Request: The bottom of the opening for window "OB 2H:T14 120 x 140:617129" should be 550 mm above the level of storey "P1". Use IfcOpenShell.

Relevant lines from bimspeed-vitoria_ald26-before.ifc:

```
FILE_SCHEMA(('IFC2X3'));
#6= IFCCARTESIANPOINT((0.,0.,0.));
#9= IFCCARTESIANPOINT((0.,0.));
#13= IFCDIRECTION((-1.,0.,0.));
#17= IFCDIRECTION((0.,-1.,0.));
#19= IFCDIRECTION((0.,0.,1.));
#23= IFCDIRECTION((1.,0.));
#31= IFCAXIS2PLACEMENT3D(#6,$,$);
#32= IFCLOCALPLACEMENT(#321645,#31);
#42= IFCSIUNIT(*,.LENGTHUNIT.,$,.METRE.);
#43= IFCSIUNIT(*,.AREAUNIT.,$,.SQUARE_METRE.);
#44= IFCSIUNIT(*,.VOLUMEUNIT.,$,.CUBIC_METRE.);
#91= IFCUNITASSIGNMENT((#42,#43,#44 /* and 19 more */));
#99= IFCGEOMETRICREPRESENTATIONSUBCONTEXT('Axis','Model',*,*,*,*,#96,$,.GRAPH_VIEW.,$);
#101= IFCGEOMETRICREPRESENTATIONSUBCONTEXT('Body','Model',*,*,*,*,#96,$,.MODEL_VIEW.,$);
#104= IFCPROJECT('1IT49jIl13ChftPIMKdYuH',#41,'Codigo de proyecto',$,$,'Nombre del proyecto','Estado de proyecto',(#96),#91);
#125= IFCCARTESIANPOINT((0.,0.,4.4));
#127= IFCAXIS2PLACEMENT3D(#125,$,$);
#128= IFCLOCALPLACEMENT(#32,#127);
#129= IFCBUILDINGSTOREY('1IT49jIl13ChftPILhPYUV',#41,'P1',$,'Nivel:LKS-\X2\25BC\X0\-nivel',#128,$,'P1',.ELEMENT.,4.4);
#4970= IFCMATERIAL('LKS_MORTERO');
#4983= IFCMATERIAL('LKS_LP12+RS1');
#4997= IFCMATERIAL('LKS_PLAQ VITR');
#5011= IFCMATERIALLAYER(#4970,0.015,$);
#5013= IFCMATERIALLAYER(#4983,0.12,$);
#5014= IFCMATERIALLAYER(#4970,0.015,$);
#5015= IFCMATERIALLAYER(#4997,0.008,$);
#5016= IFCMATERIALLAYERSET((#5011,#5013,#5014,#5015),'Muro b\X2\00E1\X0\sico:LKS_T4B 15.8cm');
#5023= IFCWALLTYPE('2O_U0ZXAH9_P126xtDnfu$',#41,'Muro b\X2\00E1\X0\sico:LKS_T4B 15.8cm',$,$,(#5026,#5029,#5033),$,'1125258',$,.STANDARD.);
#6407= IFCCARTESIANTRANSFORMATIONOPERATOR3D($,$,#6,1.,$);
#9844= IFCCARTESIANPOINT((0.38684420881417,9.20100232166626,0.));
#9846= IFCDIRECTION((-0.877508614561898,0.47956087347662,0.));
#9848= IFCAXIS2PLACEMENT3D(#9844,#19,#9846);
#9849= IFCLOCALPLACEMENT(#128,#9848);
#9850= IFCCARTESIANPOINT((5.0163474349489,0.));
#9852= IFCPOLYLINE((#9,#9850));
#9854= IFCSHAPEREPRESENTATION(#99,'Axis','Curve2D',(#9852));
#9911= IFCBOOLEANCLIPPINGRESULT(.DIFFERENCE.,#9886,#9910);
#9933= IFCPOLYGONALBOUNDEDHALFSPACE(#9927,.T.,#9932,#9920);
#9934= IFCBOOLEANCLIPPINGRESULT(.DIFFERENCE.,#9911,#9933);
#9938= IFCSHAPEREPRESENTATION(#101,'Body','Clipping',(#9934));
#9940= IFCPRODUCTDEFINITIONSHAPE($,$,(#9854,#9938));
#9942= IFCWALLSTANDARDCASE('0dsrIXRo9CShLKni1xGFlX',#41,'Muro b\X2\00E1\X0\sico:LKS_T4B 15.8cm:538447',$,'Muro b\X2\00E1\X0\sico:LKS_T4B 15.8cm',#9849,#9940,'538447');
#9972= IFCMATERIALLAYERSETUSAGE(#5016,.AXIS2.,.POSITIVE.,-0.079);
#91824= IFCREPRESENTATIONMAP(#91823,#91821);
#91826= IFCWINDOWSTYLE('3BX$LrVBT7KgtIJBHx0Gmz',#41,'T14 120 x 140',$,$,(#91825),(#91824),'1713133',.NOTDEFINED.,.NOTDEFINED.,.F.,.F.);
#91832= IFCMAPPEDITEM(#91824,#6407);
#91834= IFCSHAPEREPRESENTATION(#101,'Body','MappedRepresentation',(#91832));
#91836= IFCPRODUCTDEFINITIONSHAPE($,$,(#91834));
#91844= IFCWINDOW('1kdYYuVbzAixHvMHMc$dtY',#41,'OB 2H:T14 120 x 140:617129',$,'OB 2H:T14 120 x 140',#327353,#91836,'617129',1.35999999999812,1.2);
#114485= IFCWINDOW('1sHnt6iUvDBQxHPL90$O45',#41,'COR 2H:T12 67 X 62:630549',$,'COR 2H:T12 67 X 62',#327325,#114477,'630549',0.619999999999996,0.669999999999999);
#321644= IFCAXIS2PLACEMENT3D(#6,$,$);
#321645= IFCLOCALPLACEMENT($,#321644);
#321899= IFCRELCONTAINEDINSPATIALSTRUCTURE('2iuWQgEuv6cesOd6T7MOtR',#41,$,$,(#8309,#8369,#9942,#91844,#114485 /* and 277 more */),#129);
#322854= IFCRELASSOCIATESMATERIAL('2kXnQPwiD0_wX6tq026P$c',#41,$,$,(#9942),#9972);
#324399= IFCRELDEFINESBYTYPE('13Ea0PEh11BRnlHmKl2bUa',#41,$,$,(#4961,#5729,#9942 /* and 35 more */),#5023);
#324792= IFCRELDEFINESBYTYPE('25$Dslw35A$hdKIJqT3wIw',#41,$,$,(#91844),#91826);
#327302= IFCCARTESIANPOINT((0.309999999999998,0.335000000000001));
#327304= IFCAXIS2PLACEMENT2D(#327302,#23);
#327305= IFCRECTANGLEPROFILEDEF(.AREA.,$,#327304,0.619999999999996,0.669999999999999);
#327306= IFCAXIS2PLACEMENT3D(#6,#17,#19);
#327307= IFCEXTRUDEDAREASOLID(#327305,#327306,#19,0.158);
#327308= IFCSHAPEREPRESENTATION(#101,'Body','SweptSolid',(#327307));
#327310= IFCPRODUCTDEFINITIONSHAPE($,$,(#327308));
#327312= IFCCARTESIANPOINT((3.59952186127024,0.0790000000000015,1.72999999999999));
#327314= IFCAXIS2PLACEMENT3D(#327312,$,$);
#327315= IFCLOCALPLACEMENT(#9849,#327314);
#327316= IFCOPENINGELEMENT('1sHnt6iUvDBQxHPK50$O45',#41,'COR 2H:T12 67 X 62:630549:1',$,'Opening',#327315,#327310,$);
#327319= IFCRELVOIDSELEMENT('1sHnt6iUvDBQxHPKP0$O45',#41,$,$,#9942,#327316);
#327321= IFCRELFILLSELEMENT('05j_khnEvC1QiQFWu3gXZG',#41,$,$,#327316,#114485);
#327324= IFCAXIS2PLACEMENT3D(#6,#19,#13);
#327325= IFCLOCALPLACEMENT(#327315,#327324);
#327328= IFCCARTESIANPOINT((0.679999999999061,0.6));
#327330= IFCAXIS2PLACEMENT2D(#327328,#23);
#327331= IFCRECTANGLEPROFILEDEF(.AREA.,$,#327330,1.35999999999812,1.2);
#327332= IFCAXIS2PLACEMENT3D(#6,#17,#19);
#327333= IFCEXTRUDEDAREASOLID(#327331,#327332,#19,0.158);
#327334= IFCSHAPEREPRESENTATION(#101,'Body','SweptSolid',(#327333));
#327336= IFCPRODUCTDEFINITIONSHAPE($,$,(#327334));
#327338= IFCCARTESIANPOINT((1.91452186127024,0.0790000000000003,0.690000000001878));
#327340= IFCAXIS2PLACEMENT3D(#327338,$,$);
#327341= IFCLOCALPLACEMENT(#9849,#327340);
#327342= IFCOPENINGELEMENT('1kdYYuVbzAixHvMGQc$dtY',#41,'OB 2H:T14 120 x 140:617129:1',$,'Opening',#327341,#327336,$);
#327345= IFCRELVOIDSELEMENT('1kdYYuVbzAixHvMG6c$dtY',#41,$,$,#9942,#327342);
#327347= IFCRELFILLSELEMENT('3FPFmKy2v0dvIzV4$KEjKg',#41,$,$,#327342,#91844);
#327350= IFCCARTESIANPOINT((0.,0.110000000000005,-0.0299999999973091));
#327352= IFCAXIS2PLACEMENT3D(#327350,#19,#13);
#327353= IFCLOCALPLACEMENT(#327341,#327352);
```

```python
import numpy as np
import ifcopenshell
import ifcopenshell.api.geometry
import ifcopenshell.geom
import ifcopenshell.util.element
import ifcopenshell.util.placement
import ifcopenshell.util.shape
import ifcopenshell.util.unit

model = ifcopenshell.open("bimspeed-vitoria_ald26-before.ifc")
unit_scale = ifcopenshell.util.unit.calculate_unit_scale(model)

window = model.by_guid("1kdYYuVbzAixHvMHMc$dtY")
opening = window.FillsVoids[0].RelatingOpeningElement
storey = ifcopenshell.util.element.get_container(window, ifc_class="IfcBuildingStorey")
level = ifcopenshell.util.placement.get_local_placement(storey.ObjectPlacement)[2, 3]

# The opening's origin need not be at the sill, so measure its lowest point.
shape = ifcopenshell.geom.create_shape(ifcopenshell.geom.settings(), opening)
bottom = ifcopenshell.util.shape.get_shape_bottom_elevation(shape, shape.geometry) / unit_scale
dz = level + 0.55 - bottom

shift = np.array([0.0, 0.0, dz])
# The window is placed relative to its opening, so it follows when the opening moves.
matrix = ifcopenshell.util.placement.get_local_placement(opening.ObjectPlacement)
matrix[:3, 3] += shift
ifcopenshell.api.geometry.edit_object_placement(
    model, product=opening, matrix=matrix, is_si=False, should_transform_children=True
)

print(f"moved by {dz * unit_scale:+.3f} m")

model.write("bimspeed-vitoria_ald26-before_v2.ifc")
```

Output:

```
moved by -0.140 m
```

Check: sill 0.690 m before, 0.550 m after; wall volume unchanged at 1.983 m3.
